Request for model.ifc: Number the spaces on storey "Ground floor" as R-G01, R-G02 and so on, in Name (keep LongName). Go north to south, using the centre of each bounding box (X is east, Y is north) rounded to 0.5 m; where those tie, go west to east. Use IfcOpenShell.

First a look at what the model holds.

```python
import ifcopenshell
import ifcopenshell.util.element
import ifcopenshell.util.placement

model = ifcopenshell.open("model.ifc")
print(model.schema)
storey = next(s for s in model.by_type("IfcBuildingStorey") if s.Name == "Ground floor")
spaces = [e for e in ifcopenshell.util.element.get_decomposition(storey) if e.is_a("IfcSpace")]
for e in sorted(spaces, key=lambda e: e.id()):
    origin = ifcopenshell.util.placement.get_local_placement(e.ObjectPlacement)[:3, 3]
    print(e.id(), e.Name, e.LongName, origin.round(2) + 0.0, sep=" | ")
```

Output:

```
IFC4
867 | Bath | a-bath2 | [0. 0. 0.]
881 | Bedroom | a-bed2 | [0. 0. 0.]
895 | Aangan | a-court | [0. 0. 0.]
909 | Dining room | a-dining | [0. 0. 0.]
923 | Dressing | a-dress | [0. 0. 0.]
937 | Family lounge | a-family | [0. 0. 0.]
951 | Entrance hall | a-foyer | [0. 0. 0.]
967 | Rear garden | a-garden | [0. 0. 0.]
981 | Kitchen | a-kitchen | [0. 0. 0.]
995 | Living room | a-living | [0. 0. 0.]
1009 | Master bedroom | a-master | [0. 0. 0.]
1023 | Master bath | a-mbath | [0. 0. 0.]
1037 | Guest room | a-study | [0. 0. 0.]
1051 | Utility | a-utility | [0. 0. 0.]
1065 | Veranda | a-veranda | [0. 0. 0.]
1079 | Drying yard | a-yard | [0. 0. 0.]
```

```python
import ifcopenshell
import ifcopenshell.geom
import ifcopenshell.util.element
import ifcopenshell.util.shape

model = ifcopenshell.open("model.ifc")
settings = ifcopenshell.geom.settings()
settings.set("use-world-coords", True)


def centre(element):
    shape = ifcopenshell.geom.create_shape(settings, element)
    return ifcopenshell.util.shape.get_bbox_centroid(shape.geometry)


storey = next(s for s in model.by_type("IfcBuildingStorey") if s.Name == "Ground floor")
spaces = [e for e in ifcopenshell.util.element.get_decomposition(storey) if e.is_a("IfcSpace")]

# Insertion points can sit at a corner or the storey origin, so sort by the geometry (in metres).
centres = {e: centre(e) for e in spaces}
spaces.sort(key=lambda e: (-round(centres[e][1] / 0.5), centres[e][0]))

for i, e in enumerate(spaces, start=1):
    number = f"R-G{i:02d}"
    e.Name = number
    print(e.id(), number)

model.write("model-out.ifc")
```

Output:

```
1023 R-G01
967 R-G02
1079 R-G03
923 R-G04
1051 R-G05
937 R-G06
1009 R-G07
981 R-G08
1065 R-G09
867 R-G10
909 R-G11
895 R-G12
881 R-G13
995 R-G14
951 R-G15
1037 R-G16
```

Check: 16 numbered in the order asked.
